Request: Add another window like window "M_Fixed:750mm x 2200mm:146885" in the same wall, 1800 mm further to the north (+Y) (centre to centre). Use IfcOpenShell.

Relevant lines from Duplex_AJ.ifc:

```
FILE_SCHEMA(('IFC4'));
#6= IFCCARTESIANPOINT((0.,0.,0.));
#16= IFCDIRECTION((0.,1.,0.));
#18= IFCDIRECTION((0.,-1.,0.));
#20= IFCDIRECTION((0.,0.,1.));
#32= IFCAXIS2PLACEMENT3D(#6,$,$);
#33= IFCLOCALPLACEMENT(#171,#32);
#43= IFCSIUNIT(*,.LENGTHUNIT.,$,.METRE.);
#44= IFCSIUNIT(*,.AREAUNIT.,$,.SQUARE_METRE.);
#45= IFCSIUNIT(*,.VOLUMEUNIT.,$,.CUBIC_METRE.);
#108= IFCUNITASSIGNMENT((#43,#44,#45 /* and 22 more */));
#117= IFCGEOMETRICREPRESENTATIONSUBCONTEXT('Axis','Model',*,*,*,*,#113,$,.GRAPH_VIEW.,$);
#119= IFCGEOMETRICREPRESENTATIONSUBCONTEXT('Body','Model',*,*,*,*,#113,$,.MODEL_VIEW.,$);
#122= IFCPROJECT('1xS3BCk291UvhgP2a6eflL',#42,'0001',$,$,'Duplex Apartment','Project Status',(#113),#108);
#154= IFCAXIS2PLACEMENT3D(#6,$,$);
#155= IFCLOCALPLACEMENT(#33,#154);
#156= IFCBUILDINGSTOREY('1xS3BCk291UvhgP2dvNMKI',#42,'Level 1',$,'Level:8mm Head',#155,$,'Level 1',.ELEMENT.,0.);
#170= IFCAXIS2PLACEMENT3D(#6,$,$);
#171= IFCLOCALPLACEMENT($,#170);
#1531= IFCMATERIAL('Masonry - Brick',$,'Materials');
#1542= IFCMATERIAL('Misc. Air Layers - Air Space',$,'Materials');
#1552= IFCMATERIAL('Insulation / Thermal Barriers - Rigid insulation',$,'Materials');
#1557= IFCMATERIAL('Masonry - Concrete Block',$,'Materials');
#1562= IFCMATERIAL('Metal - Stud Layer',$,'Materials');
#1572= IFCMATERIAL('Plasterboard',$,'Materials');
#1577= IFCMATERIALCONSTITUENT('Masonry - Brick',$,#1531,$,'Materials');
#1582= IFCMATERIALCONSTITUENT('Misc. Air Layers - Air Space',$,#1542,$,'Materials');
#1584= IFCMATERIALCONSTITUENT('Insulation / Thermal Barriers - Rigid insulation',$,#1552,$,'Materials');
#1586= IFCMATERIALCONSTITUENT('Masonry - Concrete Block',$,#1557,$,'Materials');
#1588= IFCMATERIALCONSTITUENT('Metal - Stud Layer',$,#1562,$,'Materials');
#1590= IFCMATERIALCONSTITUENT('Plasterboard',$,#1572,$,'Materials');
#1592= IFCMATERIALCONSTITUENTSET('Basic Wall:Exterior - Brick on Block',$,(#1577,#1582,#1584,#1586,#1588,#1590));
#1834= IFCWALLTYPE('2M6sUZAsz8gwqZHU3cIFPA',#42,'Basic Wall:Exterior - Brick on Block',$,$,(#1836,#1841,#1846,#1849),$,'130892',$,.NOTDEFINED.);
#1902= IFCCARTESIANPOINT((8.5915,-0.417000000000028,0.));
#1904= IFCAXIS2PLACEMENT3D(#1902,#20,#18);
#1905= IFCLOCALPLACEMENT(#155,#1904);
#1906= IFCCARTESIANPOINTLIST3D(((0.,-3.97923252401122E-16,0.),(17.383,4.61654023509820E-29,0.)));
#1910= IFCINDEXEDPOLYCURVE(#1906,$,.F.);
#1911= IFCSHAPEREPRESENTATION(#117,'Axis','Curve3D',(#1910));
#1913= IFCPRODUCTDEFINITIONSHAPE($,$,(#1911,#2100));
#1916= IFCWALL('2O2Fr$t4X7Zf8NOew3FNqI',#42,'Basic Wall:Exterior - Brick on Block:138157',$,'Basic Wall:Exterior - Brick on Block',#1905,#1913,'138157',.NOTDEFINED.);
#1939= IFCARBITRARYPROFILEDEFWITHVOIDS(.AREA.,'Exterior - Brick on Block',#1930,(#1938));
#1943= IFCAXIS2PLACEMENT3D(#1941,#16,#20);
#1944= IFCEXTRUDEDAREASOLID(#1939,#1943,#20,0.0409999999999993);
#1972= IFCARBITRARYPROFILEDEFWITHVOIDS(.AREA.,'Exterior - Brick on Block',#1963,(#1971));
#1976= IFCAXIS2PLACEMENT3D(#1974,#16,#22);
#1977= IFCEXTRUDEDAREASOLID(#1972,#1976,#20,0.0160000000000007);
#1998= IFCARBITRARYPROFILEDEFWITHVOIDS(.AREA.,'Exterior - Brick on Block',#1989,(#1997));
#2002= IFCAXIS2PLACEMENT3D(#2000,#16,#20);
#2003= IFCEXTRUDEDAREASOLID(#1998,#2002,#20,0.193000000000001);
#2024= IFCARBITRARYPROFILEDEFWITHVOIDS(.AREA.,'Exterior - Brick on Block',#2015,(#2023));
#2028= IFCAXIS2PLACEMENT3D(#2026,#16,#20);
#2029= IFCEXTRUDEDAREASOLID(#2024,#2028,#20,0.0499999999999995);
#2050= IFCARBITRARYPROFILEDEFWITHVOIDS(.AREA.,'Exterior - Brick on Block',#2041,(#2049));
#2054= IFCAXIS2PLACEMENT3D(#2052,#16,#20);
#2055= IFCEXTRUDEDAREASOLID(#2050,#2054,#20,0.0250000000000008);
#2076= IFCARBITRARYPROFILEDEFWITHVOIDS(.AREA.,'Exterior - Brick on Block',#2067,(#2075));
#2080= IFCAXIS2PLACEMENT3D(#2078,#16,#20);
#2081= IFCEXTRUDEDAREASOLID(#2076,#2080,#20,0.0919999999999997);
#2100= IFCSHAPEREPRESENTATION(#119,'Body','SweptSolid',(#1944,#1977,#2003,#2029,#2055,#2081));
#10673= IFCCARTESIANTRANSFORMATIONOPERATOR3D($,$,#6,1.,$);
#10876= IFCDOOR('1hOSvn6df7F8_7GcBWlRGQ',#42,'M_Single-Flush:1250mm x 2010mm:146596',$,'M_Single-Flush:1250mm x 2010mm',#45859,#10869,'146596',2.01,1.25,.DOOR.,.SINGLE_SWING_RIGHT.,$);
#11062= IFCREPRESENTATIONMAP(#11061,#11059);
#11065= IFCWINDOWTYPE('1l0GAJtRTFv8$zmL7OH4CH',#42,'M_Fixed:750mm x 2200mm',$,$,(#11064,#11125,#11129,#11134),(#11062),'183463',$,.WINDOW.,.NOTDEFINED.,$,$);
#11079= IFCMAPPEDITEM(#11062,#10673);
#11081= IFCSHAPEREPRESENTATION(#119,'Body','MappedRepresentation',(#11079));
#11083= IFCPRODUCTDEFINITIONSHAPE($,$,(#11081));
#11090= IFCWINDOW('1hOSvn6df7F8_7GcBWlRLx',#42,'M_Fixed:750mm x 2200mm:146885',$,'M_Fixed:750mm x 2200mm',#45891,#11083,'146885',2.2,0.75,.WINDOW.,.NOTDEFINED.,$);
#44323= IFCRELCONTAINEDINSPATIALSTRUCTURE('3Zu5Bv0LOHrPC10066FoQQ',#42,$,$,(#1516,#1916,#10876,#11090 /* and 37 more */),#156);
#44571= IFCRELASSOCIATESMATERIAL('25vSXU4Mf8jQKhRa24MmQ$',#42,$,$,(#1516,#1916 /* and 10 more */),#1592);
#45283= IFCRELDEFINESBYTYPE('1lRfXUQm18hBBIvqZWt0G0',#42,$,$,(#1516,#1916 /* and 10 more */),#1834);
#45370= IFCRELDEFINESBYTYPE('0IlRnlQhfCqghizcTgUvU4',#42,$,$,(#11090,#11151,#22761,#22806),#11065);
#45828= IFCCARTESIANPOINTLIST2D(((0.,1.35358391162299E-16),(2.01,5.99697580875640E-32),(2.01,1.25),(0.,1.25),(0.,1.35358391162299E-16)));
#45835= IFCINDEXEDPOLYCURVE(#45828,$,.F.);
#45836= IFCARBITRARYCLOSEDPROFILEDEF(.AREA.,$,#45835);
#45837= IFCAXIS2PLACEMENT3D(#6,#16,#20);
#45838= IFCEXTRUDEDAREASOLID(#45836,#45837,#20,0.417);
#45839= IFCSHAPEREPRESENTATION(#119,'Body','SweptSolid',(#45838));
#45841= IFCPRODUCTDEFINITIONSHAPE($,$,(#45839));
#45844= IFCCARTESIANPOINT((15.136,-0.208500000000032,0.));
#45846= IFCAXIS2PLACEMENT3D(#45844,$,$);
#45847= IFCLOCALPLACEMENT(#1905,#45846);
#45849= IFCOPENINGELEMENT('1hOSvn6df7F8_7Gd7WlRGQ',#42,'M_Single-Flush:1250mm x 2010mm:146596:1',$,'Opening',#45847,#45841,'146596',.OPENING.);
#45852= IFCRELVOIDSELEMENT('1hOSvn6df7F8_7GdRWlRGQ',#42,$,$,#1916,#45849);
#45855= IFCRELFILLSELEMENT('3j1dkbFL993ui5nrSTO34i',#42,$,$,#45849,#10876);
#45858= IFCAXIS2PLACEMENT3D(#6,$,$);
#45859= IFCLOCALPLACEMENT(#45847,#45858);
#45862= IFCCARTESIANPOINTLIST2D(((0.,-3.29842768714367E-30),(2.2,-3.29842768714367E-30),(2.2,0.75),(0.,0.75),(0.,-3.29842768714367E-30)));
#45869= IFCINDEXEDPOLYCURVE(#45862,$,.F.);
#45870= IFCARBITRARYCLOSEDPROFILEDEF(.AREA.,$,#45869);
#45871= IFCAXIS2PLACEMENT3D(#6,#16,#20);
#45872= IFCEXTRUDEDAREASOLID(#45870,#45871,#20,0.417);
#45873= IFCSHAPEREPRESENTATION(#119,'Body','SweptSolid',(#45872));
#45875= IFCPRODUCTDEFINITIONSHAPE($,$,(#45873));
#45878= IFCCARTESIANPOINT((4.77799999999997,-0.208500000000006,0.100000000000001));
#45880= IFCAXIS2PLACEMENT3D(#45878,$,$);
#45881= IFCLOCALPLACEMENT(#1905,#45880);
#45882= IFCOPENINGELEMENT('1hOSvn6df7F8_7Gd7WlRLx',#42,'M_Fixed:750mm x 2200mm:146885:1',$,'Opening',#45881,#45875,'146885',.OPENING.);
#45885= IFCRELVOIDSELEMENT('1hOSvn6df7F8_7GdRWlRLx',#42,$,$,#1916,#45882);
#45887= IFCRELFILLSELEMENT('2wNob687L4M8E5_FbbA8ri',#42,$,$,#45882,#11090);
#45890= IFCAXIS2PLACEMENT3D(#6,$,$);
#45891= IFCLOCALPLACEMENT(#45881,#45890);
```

```python
import ifcopenshell
import ifcopenshell.api.feature
import ifcopenshell.api.geometry
import ifcopenshell.api.root
import ifcopenshell.geom
import ifcopenshell.util.element
import ifcopenshell.util.placement
import ifcopenshell.util.shape
import ifcopenshell.util.unit

model = ifcopenshell.open("Duplex_AJ.ifc")
unit_scale = ifcopenshell.util.unit.calculate_unit_scale(model)
settings = ifcopenshell.geom.settings()


def volume(element):
    """Net volume in cubic metres, openings subtracted."""
    shape = ifcopenshell.geom.create_shape(settings, element)
    return ifcopenshell.util.shape.get_volume(shape.geometry)


def reuse_history(source, copy):
    """copy_class also copies each property set's owner history, people and application; keep the originals."""
    for rel in copy.IsDefinedBy:
        if rel.is_a("IfcRelDefinesByProperties") and (history := rel.RelatingPropertyDefinition.OwnerHistory):
            rel.RelatingPropertyDefinition.OwnerHistory = source.OwnerHistory
            ifcopenshell.util.element.remove_deep2(model, history)


window = model.by_id(11090)
opening = window.FillsVoids[0].RelatingOpeningElement
wall = opening.VoidsElements[0].RelatingBuildingElement
before = volume(wall)
shift = ifcopenshell.util.placement.get_local_placement(wall.ObjectPlacement)[:3, 0] * -1.8 / unit_scale

# copy_class copies the void relationship, type, container and properties, but no geometry.
new_opening = ifcopenshell.api.root.copy_class(model, product=opening)
new_opening.Representation = ifcopenshell.util.element.copy_deep(
    model, opening.Representation, exclude=["IfcGeometricRepresentationContext", "IfcRepresentationMap"]
)
new_opening.Name = "M_Fixed:750mm x 2200mm"
new_opening.Tag = None
new_window = ifcopenshell.api.root.copy_class(model, product=window)
new_window.Representation = ifcopenshell.util.element.copy_deep(
    model, window.Representation, exclude=["IfcGeometricRepresentationContext", "IfcRepresentationMap"]
)
new_window.Name = "M_Fixed:750mm x 2200mm"
new_window.Tag = None
reuse_history(window, new_window)
ifcopenshell.api.feature.add_filling(model, opening=new_opening, element=new_window)

for old, new in ((opening, new_opening), (window, new_window)):
    matrix = ifcopenshell.util.placement.get_local_placement(old.ObjectPlacement)
    matrix[:3, 3] += shift
    ifcopenshell.api.geometry.edit_object_placement(model, product=new, matrix=matrix, is_si=False)

after = volume(wall)

print(f"wall volume {before:.3f} -> {after:.3f} m3")

model.write("Duplex_AJ_updated.ifc")
```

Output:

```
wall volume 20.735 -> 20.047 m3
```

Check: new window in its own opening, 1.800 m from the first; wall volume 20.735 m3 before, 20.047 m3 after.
